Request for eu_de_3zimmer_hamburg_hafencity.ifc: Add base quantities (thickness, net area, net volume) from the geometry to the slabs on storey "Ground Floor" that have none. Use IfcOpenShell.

First a look at what the model holds.

```python
import ifcopenshell
import ifcopenshell.util.element
import ifcopenshell.util.unit

model = ifcopenshell.open("eu_de_3zimmer_hamburg_hafencity.ifc")
print(model.schema)
for unit_type in ("LENGTHUNIT", "AREAUNIT", "VOLUMEUNIT"):
    print(unit_type, ifcopenshell.util.unit.calculate_unit_scale(model, unit_type))
storey = next(s for s in model.by_type("IfcBuildingStorey") if s.Name == "Ground Floor")
slabs = [e for e in ifcopenshell.util.element.get_decomposition(storey) if e.is_a("IfcSlab")]
for e in sorted(slabs, key=lambda e: e.id()):
    print(e.id(), e.is_a(), e.Name, list(ifcopenshell.util.element.get_psets(e, qtos_only=True)), sep=" | ")
```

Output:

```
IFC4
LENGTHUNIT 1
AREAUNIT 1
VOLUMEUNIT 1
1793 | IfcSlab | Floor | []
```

```python
import ifcopenshell
import ifcopenshell.api.pset
import ifcopenshell.geom
import ifcopenshell.util.element
import ifcopenshell.util.shape
import ifcopenshell.util.unit

model = ifcopenshell.open("eu_de_3zimmer_hamburg_hafencity.ifc")
unit_scale = ifcopenshell.util.unit.calculate_unit_scale(model)
area_scale = ifcopenshell.util.unit.calculate_unit_scale(model, "AREAUNIT")
volume_scale = ifcopenshell.util.unit.calculate_unit_scale(model, "VOLUMEUNIT")
settings = ifcopenshell.geom.settings()

storey = next(s for s in model.by_type("IfcBuildingStorey") if s.Name == "Ground Floor")
slabs = [e for e in ifcopenshell.util.element.get_decomposition(storey) if e.is_a("IfcSlab")]

for e in sorted(slabs, key=lambda e: e.id()):
    if ifcopenshell.util.element.get_psets(e, qtos_only=True, should_inherit=False):
        continue
    # Geometry comes back in metres, in the element's own axes.
    shape = ifcopenshell.geom.create_shape(settings, e)
    values = {
        "Width": ifcopenshell.util.shape.get_z(shape.geometry) / unit_scale,
        "NetArea": ifcopenshell.util.shape.get_footprint_area(shape.geometry) / area_scale,
        "NetVolume": ifcopenshell.util.shape.get_volume(shape.geometry) / volume_scale,
    }
    qto = ifcopenshell.api.pset.add_qto(model, product=e, name="Qto_SlabBaseQuantities")
    ifcopenshell.api.pset.edit_qto(model, qto=qto, properties=values)
    print(e.id(), {k: round(v, 3) for k, v in values.items()})

model.write("eu_de_3zimmer_hamburg_hafencity_edited.ifc")
```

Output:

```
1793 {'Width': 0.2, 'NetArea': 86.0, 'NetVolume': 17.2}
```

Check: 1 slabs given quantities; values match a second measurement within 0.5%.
